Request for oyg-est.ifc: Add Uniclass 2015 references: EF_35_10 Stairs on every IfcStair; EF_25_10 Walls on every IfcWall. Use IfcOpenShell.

First a look at what the model holds.

```python
import ifcopenshell

model = ifcopenshell.open("oyg-est.ifc")
print(model.schema)
print("classifications:", [c.Name for c in model.by_type("IfcClassification")])
for ifc_class in ("IfcDoor", "IfcRoof", "IfcStair", "IfcWall", "IfcWindow"):
    print(ifc_class, len(model.by_type(ifc_class)))
```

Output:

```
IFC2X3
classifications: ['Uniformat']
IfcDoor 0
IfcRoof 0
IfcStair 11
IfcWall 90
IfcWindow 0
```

```python
import ifcopenshell
import ifcopenshell.api.classification

model = ifcopenshell.open("oyg-est.ifc")

# IFC2X3 requires Source and Edition and has no link from the project to the system.
system = model.create_entity("IfcClassification", Source="NBS", Edition="2015", Name="Uniclass 2015")

codes = {
    "IfcStair": ("EF_35_10", "Stairs"),
    "IfcWall": ("EF_25_10", "Walls"),
}
for ifc_class, (code, name) in codes.items():
    products = model.by_type(ifc_class)
    ifcopenshell.api.classification.add_reference(
        model, products=products, classification=system, identification=code, name=name
    )
    print(code, len(products))

model.write("oyg-est_updated.ifc")
```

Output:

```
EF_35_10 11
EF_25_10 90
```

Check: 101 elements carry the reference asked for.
